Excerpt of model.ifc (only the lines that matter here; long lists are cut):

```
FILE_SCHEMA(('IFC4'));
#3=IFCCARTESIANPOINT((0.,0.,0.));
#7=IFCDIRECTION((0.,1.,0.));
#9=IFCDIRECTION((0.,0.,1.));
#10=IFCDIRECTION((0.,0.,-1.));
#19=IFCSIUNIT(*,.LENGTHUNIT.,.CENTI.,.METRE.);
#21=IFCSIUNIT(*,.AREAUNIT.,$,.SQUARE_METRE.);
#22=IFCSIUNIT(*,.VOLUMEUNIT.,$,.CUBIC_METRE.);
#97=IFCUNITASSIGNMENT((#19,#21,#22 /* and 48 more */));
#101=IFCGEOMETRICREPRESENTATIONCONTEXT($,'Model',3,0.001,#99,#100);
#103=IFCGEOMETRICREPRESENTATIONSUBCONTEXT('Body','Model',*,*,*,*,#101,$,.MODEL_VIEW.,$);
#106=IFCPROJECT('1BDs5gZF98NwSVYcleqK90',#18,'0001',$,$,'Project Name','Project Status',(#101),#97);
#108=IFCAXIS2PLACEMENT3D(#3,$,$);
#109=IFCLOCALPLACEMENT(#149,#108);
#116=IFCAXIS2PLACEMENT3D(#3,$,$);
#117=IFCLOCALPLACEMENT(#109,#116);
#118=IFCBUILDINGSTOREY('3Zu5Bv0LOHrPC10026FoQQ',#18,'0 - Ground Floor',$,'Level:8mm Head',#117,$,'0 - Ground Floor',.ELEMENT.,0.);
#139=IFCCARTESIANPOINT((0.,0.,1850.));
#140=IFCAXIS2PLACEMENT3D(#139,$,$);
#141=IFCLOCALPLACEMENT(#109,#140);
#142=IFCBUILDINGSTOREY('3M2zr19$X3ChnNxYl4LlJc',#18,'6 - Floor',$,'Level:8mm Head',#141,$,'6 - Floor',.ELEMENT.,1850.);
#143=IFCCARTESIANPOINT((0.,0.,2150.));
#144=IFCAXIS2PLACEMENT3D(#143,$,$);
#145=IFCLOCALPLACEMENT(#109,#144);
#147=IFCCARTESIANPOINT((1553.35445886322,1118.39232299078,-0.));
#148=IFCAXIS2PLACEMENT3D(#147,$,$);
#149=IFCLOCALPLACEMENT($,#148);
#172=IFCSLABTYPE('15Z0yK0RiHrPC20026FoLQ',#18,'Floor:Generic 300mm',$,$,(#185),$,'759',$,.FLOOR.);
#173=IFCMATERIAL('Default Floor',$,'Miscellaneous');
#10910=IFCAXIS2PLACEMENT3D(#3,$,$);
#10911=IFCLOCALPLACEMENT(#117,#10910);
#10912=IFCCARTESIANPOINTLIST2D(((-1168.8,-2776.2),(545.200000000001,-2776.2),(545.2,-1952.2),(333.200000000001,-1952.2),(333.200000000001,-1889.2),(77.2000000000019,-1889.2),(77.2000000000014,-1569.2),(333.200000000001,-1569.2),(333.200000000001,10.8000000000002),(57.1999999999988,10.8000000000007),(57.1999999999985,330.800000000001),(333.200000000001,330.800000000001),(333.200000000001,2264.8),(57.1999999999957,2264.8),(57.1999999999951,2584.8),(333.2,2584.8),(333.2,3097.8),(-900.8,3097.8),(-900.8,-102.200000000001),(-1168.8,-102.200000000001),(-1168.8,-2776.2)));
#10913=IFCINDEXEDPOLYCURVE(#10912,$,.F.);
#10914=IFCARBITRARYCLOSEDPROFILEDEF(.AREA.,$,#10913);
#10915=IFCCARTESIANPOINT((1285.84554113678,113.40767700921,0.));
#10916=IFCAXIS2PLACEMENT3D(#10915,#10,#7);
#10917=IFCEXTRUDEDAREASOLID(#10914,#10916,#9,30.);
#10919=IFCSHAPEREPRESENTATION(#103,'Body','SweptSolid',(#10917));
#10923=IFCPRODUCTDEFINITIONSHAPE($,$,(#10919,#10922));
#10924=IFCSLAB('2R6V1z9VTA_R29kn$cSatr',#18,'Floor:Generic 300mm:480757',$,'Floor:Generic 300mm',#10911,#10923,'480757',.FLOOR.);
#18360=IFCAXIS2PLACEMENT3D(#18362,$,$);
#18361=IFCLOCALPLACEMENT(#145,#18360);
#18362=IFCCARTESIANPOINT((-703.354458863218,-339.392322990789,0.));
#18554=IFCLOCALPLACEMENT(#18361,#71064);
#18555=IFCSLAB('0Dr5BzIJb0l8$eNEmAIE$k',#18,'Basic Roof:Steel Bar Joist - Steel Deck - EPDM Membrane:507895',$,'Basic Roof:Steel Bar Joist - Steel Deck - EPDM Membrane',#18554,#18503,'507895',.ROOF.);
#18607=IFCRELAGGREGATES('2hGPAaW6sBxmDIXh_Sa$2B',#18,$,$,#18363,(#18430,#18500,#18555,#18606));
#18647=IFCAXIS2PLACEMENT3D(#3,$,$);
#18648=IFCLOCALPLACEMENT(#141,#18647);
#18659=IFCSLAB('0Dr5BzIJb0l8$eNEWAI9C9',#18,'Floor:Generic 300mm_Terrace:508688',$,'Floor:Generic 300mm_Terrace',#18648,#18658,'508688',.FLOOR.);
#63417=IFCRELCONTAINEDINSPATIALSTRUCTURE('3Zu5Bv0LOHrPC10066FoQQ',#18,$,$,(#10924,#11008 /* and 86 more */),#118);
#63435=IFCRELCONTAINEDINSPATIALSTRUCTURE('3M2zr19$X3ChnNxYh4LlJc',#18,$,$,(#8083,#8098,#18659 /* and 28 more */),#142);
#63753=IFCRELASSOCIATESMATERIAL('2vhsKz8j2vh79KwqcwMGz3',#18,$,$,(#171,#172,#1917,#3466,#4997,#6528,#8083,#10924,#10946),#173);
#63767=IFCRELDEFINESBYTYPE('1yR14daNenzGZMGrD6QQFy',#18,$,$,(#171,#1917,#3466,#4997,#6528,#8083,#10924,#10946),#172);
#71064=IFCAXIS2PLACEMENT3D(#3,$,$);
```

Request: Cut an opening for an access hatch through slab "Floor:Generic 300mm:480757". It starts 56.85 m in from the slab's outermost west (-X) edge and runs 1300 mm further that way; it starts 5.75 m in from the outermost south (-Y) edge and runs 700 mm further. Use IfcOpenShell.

```python
import numpy as np
import ifcopenshell
import ifcopenshell.api.feature
import ifcopenshell.api.geometry
import ifcopenshell.api.root
import ifcopenshell.geom
import ifcopenshell.util.placement
import ifcopenshell.util.representation
import ifcopenshell.util.shape
import ifcopenshell.util.unit

model = ifcopenshell.open("model.ifc")
unit_scale = ifcopenshell.util.unit.calculate_unit_scale(model)
settings = ifcopenshell.geom.settings()


def volume(element):
    """Net volume in cubic metres, openings subtracted."""
    shape = ifcopenshell.geom.create_shape(settings, element)
    return ifcopenshell.util.shape.get_volume(shape.geometry)


slab = model.by_guid("2R6V1z9VTA_R29kn$cSatr")
before = volume(slab)

# Extent in the slab's own axes, in metres. The edges named are its -X and -Y sides.
slab_shape = ifcopenshell.geom.create_shape(settings, slab)
vertices = ifcopenshell.util.shape.get_vertices(slab_shape.geometry)
x_min, y_min, bottom = vertices.min(axis=0)
top = vertices[:, 2].max()

opening = ifcopenshell.api.root.create_entity(model, ifc_class="IfcOpeningElement", name="Access hatch opening", predefined_type="OPENING")
context = ifcopenshell.util.representation.get_context(model, "Model", "Body", "MODEL_VIEW")
width, depth = 1.3, 0.7
outline = [(0.0, 0.0), (width, 0.0), (width, depth), (0.0, depth), (0.0, 0.0)]
# Overshoot both faces by 50 mm so the cut is clean.
shape = ifcopenshell.api.geometry.add_slab_representation(
    model, context=context, depth=top - bottom + 0.1, polyline=outline
)
ifcopenshell.api.geometry.assign_representation(model, product=opening, representation=shape)

matrix = ifcopenshell.util.placement.get_local_placement(slab.ObjectPlacement)
matrix[:, 3] = matrix @ np.append(np.array([x_min + 56.85, y_min + 5.75, bottom - 0.05]) / unit_scale, 1.0)
ifcopenshell.api.geometry.edit_object_placement(model, product=opening, matrix=matrix, is_si=False)
ifcopenshell.api.feature.add_feature(model, feature=opening, element=slab)

after = volume(slab)

print(f"slab volume {before:.3f} -> {after:.3f} m3")

model.write("model_edited.ifc")
```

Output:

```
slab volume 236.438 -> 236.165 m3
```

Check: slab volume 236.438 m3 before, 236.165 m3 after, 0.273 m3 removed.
